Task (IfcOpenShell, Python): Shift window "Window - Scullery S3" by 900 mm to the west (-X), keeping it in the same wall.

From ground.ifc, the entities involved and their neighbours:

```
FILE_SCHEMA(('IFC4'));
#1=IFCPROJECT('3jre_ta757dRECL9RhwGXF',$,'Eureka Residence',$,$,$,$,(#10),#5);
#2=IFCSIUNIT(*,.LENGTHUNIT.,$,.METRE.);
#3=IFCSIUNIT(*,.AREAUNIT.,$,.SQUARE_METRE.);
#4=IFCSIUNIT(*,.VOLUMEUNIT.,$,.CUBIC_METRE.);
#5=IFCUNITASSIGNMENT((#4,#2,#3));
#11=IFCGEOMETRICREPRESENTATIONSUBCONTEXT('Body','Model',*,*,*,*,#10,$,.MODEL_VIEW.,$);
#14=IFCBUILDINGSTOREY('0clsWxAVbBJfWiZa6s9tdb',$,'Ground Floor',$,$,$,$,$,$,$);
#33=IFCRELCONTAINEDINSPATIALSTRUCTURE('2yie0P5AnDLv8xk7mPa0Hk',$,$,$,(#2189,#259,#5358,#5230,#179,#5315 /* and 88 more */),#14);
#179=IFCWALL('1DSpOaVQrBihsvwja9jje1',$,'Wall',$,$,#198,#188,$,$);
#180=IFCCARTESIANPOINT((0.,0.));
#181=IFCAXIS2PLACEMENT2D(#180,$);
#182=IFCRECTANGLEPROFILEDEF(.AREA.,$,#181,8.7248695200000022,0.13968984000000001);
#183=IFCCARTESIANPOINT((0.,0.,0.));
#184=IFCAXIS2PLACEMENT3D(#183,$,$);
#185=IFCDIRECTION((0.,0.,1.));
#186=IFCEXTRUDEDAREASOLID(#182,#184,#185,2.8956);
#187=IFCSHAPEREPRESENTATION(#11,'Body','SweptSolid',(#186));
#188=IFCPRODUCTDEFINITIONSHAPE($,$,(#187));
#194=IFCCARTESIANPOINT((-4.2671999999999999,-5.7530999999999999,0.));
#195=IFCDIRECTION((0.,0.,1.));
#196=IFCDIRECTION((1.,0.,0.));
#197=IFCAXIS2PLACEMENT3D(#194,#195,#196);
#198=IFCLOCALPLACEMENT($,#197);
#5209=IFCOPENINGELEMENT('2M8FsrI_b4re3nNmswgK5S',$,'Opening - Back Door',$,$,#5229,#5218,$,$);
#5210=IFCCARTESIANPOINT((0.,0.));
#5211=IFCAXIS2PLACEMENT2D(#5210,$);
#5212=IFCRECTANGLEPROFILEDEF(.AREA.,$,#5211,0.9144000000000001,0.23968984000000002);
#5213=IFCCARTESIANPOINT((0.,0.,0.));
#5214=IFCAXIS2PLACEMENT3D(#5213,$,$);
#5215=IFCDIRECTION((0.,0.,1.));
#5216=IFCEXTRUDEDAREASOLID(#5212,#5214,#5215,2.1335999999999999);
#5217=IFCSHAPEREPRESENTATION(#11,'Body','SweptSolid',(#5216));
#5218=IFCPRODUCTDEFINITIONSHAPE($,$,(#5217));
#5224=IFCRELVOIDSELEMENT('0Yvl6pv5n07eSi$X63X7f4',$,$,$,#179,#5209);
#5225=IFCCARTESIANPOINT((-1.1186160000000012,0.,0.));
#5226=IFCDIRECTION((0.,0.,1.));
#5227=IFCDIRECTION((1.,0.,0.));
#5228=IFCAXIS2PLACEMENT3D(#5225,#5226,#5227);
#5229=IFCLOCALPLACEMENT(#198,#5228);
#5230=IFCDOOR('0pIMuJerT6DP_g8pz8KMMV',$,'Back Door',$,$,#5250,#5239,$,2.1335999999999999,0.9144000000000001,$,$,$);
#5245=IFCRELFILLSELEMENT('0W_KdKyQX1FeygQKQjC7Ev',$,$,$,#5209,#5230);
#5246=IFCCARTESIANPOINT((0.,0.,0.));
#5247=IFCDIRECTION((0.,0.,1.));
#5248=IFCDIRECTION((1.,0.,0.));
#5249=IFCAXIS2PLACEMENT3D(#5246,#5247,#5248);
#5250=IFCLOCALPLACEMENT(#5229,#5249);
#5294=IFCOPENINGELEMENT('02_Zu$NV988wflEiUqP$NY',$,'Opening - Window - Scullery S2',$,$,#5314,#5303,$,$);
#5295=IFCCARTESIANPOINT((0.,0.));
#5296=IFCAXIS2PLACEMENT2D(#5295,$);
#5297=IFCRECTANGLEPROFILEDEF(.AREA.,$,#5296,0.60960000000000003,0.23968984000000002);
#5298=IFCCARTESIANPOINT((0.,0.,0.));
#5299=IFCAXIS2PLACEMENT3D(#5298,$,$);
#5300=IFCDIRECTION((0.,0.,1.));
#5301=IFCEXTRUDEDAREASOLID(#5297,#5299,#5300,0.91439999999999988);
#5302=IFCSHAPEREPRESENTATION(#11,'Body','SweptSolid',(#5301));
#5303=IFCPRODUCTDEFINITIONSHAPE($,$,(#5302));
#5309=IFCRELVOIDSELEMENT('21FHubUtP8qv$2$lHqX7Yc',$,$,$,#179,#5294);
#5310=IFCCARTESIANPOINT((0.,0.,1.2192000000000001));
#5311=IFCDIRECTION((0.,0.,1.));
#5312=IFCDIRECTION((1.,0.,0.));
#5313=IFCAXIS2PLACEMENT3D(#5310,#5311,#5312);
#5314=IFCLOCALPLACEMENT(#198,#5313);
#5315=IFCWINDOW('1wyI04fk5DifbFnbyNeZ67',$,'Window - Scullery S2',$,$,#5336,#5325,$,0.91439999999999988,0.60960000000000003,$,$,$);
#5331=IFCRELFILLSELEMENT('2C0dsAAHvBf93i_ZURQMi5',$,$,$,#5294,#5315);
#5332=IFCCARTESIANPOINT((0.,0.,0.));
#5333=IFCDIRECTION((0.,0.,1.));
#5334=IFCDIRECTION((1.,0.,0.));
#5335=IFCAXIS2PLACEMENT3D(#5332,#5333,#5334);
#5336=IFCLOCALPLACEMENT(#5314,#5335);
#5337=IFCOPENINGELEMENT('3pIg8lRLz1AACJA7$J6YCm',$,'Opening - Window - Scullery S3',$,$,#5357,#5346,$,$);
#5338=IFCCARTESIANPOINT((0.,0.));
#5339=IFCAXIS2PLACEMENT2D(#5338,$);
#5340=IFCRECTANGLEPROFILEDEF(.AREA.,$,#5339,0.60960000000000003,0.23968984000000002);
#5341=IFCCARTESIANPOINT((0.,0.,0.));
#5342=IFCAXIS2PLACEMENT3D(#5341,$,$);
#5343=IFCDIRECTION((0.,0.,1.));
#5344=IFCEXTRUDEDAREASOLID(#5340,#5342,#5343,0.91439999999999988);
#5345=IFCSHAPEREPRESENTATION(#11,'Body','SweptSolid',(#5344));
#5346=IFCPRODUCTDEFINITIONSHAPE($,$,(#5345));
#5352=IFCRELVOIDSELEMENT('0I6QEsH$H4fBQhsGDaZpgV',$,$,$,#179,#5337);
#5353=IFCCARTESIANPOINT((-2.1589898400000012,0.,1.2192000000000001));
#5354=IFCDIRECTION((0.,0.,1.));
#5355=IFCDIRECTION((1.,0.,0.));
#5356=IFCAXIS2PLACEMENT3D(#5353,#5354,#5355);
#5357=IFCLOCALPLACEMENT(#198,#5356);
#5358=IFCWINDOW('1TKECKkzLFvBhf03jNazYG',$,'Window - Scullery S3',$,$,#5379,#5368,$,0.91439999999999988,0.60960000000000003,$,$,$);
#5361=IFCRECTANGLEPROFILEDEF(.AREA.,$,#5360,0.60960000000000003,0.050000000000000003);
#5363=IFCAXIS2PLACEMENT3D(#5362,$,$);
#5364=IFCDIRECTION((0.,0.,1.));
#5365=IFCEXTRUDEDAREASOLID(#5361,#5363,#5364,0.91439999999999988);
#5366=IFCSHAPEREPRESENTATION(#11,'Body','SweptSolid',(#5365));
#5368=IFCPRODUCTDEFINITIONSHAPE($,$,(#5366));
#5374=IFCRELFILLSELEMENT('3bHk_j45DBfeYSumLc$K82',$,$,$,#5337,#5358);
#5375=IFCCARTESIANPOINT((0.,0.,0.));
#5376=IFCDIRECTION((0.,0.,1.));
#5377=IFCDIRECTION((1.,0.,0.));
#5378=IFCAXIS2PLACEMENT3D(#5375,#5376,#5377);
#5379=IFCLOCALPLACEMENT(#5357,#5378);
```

```python
import ifcopenshell
import ifcopenshell.api.geometry
import ifcopenshell.util.placement
import ifcopenshell.util.unit

model = ifcopenshell.open("ground.ifc")
unit_scale = ifcopenshell.util.unit.calculate_unit_scale(model)

window = model.by_guid("1TKECKkzLFvBhf03jNazYG")
opening = window.FillsVoids[0].RelatingOpeningElement
wall = opening.VoidsElements[0].RelatingBuildingElement

wall_matrix = ifcopenshell.util.placement.get_local_placement(wall.ObjectPlacement)
shift = wall_matrix[:3, 0] * -0.9 / unit_scale
before = ifcopenshell.util.placement.get_local_placement(window.ObjectPlacement)[:3, 3].copy()

# The window is placed relative to its opening, so it follows when the opening moves.
matrix = ifcopenshell.util.placement.get_local_placement(opening.ObjectPlacement)
matrix[:3, 3] += shift
ifcopenshell.api.geometry.edit_object_placement(
    model, product=opening, matrix=matrix, is_si=False, should_transform_children=True
)

after = ifcopenshell.util.placement.get_local_placement(window.ObjectPlacement)[:3, 3]
print("window moved by", (after - before).round(3) + 0.0)

model.write("ground_v2.ifc")
```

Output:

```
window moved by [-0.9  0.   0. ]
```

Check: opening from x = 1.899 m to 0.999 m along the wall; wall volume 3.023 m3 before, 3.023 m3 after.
